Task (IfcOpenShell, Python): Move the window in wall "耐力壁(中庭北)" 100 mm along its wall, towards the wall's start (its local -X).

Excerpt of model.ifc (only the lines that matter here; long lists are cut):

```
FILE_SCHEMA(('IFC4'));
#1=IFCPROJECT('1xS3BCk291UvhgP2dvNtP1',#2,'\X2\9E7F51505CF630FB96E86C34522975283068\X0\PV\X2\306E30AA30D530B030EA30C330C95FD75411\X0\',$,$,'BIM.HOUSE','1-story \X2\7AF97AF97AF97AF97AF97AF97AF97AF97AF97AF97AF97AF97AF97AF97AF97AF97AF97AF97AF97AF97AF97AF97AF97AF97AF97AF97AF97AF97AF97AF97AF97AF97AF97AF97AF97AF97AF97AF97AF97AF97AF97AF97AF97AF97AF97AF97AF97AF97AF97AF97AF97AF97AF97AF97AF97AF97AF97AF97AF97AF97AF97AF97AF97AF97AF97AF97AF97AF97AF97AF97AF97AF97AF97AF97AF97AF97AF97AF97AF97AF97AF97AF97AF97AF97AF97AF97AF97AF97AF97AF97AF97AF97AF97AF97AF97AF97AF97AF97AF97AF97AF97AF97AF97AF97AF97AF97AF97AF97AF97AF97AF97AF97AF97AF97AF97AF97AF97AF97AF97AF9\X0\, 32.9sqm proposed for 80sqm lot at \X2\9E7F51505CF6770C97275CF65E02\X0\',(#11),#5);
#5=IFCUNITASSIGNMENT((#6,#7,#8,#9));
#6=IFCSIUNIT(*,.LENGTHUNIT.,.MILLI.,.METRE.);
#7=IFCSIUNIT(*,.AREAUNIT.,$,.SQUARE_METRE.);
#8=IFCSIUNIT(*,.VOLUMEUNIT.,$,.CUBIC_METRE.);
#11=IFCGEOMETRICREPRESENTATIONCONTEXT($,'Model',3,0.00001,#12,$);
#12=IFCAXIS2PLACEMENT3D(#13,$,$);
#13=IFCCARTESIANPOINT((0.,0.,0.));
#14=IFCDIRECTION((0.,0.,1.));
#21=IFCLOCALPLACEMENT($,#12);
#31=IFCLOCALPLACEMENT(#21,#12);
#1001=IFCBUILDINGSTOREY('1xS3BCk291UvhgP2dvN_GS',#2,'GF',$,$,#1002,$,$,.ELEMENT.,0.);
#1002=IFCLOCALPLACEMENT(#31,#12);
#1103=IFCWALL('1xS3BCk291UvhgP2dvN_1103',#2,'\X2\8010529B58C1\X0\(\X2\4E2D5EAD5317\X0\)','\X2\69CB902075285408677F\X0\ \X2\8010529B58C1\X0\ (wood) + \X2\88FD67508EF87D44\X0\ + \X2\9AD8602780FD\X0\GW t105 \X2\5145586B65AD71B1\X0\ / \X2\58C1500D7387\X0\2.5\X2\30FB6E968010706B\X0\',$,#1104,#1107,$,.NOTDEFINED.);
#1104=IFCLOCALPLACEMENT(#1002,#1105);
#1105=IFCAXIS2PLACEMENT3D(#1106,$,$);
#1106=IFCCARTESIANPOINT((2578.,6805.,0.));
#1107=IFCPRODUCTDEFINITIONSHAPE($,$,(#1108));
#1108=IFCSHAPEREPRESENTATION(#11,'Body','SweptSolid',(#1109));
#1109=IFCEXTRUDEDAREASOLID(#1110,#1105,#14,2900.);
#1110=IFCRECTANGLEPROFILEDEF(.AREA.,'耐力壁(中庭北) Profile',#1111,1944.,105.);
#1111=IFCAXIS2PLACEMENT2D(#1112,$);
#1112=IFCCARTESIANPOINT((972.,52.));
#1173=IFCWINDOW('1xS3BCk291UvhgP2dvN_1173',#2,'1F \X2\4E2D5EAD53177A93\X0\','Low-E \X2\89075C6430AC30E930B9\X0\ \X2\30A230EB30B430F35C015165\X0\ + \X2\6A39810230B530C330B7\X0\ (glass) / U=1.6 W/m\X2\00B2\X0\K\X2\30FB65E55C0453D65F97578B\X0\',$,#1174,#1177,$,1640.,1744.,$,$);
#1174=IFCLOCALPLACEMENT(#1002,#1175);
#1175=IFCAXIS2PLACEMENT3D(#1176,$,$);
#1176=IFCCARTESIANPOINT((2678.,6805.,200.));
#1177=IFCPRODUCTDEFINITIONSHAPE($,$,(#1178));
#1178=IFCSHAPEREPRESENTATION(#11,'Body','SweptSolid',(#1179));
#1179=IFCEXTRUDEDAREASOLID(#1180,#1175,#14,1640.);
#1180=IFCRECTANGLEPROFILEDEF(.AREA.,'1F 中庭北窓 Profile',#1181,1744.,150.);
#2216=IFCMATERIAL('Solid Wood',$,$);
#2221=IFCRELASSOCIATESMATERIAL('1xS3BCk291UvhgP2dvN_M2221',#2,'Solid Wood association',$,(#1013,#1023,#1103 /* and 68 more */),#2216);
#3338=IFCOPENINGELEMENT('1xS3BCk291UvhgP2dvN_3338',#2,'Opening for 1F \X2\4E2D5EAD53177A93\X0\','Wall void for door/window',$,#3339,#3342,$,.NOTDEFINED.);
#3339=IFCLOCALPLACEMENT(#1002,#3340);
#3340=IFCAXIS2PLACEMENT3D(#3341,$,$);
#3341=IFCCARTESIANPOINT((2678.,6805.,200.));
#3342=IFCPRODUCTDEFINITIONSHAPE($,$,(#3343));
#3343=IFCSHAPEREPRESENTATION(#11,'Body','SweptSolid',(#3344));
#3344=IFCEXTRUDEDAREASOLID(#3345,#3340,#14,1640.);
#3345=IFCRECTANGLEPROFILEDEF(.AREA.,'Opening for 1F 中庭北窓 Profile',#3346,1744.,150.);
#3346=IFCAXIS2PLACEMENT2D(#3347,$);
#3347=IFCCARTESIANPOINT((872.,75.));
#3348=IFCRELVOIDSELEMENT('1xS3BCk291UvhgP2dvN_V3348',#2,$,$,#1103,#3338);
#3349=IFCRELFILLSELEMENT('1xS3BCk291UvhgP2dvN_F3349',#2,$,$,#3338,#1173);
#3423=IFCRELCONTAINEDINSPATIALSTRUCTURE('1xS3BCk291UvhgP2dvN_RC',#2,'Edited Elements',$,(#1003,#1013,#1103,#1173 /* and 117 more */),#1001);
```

```python
import ifcopenshell
import ifcopenshell.api.geometry
import ifcopenshell.util.placement
import ifcopenshell.util.unit

model = ifcopenshell.open("model.ifc")
unit_scale = ifcopenshell.util.unit.calculate_unit_scale(model)

window = model.by_id(1173)
opening = window.FillsVoids[0].RelatingOpeningElement
wall = opening.VoidsElements[0].RelatingBuildingElement

wall_matrix = ifcopenshell.util.placement.get_local_placement(wall.ObjectPlacement)
shift = wall_matrix[:3, 0] * -0.1 / unit_scale
before = ifcopenshell.util.placement.get_local_placement(window.ObjectPlacement)[:3, 3].copy()

# The window is not placed relative to its opening, so move both.
for product in (opening, window):
    matrix = ifcopenshell.util.placement.get_local_placement(product.ObjectPlacement)
    matrix[:3, 3] += shift
    ifcopenshell.api.geometry.edit_object_placement(model, product=product, matrix=matrix, is_si=False)

after = ifcopenshell.util.placement.get_local_placement(window.ObjectPlacement)[:3, 3]
print("window moved by", (after - before).round(3) + 0.0)

model.write("model_updated.ifc")
```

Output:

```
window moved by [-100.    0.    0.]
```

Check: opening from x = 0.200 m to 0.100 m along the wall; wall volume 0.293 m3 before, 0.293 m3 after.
